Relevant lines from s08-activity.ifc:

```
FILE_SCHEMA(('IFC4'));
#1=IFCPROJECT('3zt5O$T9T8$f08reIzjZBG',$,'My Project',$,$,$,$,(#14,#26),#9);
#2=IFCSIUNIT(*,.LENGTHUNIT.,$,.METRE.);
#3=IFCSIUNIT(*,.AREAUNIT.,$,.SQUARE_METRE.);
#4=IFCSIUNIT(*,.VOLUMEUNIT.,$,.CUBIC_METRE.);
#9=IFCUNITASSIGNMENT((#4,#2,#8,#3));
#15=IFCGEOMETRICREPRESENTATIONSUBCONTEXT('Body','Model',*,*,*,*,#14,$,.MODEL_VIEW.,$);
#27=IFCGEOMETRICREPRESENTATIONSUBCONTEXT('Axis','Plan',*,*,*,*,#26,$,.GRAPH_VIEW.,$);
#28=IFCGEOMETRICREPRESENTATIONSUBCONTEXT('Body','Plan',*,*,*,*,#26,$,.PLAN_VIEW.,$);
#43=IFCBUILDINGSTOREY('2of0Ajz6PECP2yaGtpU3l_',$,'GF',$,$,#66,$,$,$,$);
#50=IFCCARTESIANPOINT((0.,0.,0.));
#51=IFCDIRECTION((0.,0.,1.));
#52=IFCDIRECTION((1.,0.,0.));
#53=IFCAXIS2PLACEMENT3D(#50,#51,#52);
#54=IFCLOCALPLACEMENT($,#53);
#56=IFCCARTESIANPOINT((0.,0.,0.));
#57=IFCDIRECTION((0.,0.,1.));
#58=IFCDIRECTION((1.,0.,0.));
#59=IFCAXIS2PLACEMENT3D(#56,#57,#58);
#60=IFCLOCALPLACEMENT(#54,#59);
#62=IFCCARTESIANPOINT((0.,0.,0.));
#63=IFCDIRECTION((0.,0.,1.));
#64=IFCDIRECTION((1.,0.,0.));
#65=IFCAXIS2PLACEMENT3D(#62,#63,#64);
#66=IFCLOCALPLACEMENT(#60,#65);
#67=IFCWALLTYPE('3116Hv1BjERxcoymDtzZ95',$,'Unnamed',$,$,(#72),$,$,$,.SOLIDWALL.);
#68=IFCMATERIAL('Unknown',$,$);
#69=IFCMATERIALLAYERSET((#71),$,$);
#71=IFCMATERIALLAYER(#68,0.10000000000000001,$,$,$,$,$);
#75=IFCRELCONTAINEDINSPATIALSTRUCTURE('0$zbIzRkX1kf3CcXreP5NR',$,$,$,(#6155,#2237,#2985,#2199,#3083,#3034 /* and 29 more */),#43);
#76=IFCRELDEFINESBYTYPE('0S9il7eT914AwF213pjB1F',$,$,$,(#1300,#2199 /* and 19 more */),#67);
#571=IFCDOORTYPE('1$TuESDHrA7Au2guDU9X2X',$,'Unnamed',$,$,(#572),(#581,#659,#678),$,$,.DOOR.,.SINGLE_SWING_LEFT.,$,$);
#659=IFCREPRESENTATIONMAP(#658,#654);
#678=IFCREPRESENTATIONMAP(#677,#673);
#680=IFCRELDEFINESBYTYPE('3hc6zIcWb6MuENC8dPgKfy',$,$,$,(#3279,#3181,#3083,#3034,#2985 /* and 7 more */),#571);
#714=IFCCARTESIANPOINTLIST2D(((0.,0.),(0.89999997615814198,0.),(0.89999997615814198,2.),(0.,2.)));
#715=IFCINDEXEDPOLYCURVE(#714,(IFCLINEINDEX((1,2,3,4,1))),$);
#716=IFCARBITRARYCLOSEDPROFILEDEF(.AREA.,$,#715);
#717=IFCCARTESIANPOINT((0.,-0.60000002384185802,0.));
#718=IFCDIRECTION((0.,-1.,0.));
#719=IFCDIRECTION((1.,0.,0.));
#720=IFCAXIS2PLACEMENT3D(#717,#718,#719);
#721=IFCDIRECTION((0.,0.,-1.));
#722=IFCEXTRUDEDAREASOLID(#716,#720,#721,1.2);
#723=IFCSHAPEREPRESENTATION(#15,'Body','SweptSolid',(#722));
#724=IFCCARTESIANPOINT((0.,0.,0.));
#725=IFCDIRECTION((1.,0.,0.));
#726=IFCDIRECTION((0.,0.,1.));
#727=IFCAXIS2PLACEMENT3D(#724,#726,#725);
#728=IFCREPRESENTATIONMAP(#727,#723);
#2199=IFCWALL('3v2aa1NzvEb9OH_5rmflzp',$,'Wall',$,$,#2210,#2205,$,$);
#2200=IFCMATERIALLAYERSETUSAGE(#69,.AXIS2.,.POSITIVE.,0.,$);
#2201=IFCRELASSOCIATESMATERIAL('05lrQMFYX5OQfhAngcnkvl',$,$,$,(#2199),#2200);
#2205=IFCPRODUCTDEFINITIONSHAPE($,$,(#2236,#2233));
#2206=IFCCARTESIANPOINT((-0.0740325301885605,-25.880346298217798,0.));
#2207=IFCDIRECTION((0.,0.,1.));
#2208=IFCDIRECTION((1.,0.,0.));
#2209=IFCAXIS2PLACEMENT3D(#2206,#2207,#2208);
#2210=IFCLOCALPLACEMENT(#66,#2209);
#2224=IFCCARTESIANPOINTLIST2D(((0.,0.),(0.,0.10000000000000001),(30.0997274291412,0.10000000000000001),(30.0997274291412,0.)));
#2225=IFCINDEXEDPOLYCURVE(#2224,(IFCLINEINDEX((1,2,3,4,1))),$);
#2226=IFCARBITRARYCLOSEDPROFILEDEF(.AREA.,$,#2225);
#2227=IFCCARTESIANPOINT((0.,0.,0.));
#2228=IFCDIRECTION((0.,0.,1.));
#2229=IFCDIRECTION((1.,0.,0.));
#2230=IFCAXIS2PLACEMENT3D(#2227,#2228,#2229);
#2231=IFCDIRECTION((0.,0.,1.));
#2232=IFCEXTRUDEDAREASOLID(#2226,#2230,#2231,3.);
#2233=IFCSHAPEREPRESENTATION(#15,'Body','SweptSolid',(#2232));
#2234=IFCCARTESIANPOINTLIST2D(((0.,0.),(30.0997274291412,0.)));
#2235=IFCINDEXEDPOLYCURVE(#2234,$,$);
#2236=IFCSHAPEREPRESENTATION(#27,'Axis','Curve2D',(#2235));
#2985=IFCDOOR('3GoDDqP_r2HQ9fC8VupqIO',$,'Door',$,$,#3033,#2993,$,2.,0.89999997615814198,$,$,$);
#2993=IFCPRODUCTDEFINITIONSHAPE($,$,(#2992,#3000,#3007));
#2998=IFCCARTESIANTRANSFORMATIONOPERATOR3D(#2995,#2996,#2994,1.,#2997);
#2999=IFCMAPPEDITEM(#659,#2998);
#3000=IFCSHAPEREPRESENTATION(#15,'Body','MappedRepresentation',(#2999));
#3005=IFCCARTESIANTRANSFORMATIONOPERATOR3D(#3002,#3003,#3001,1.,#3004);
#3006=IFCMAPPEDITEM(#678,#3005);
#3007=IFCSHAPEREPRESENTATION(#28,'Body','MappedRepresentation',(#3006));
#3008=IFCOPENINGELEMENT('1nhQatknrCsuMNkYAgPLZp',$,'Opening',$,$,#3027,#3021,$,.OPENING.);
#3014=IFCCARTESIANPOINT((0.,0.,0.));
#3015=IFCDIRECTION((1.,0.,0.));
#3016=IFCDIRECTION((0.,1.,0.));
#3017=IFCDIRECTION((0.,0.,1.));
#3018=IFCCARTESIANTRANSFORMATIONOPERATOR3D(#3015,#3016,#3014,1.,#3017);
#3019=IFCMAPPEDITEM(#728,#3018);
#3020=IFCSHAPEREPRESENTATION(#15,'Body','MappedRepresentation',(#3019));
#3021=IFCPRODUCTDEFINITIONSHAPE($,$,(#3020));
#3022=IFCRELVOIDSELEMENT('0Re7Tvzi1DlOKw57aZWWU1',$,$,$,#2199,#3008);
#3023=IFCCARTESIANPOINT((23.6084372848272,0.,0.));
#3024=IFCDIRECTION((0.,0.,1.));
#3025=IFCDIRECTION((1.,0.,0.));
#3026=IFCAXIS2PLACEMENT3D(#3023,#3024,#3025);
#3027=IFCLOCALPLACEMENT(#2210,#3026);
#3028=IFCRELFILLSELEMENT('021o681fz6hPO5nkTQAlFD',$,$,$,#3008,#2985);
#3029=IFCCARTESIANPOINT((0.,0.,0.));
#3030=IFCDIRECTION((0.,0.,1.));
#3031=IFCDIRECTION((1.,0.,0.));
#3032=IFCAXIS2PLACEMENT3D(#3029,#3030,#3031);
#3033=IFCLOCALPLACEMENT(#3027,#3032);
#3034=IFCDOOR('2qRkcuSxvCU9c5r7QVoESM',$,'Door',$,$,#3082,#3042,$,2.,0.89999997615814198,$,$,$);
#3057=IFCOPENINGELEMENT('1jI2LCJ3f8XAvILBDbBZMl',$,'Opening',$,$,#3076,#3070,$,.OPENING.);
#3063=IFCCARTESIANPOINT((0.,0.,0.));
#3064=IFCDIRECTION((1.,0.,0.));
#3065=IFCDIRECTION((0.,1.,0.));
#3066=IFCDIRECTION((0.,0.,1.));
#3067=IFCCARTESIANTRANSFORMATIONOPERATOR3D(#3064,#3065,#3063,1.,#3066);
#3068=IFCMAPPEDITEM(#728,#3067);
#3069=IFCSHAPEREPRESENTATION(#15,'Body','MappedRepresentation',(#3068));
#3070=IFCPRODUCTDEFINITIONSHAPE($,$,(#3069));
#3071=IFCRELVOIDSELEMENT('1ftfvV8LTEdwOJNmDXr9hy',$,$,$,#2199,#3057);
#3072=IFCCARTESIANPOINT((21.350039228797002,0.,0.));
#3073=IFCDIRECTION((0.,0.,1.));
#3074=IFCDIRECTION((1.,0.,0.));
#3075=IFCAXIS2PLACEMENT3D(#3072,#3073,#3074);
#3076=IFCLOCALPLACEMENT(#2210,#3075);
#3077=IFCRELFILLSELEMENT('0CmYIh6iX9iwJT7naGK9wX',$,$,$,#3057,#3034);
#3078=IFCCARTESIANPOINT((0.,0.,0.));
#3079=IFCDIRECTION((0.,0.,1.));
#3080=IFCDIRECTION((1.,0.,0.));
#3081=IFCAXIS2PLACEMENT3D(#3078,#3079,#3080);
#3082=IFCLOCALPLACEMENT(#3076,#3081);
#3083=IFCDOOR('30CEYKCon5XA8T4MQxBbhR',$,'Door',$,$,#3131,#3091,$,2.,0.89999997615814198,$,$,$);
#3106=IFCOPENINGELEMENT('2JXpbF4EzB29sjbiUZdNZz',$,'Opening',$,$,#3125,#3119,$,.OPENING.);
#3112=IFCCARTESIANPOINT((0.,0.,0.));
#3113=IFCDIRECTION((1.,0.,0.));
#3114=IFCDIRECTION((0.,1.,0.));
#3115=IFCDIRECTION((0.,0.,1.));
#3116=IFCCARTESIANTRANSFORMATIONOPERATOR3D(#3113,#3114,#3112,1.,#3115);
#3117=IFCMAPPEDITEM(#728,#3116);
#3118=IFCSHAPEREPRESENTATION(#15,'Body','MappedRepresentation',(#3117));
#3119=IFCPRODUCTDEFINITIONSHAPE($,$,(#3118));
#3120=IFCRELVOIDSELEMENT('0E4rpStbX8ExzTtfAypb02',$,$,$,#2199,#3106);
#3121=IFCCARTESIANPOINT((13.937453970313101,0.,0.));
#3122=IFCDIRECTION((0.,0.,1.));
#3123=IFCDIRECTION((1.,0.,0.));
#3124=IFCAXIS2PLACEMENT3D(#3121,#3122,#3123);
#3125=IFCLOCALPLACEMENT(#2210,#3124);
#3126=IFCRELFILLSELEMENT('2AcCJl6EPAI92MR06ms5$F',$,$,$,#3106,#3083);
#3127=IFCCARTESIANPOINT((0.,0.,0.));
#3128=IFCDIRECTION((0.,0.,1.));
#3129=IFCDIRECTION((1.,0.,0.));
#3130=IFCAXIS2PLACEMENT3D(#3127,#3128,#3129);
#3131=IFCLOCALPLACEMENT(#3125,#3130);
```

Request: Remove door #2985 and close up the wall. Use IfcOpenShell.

```python
import ifcopenshell
import ifcopenshell.api.feature
import ifcopenshell.api.root
import ifcopenshell.geom
import ifcopenshell.util.shape

model = ifcopenshell.open("s08-activity.ifc")
settings = ifcopenshell.geom.settings()


def volume(element):
    """Net volume in cubic metres, openings subtracted."""
    shape = ifcopenshell.geom.create_shape(settings, element)
    return ifcopenshell.util.shape.get_volume(shape.geometry)


door = model.by_guid("3GoDDqP_r2HQ9fC8VupqIO")
opening = door.FillsVoids[0].RelatingOpeningElement
wall = opening.VoidsElements[0].RelatingBuildingElement
before = volume(wall)

ifcopenshell.api.root.remove_product(model, product=door)
ifcopenshell.api.feature.remove_feature(model, feature=opening)

after = volume(wall)

print(f"wall volume {before:.3f} -> {after:.3f} m3")

model.write("s08-activity_v2.ifc")
```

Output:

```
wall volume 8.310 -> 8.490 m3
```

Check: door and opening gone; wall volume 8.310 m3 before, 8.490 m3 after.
